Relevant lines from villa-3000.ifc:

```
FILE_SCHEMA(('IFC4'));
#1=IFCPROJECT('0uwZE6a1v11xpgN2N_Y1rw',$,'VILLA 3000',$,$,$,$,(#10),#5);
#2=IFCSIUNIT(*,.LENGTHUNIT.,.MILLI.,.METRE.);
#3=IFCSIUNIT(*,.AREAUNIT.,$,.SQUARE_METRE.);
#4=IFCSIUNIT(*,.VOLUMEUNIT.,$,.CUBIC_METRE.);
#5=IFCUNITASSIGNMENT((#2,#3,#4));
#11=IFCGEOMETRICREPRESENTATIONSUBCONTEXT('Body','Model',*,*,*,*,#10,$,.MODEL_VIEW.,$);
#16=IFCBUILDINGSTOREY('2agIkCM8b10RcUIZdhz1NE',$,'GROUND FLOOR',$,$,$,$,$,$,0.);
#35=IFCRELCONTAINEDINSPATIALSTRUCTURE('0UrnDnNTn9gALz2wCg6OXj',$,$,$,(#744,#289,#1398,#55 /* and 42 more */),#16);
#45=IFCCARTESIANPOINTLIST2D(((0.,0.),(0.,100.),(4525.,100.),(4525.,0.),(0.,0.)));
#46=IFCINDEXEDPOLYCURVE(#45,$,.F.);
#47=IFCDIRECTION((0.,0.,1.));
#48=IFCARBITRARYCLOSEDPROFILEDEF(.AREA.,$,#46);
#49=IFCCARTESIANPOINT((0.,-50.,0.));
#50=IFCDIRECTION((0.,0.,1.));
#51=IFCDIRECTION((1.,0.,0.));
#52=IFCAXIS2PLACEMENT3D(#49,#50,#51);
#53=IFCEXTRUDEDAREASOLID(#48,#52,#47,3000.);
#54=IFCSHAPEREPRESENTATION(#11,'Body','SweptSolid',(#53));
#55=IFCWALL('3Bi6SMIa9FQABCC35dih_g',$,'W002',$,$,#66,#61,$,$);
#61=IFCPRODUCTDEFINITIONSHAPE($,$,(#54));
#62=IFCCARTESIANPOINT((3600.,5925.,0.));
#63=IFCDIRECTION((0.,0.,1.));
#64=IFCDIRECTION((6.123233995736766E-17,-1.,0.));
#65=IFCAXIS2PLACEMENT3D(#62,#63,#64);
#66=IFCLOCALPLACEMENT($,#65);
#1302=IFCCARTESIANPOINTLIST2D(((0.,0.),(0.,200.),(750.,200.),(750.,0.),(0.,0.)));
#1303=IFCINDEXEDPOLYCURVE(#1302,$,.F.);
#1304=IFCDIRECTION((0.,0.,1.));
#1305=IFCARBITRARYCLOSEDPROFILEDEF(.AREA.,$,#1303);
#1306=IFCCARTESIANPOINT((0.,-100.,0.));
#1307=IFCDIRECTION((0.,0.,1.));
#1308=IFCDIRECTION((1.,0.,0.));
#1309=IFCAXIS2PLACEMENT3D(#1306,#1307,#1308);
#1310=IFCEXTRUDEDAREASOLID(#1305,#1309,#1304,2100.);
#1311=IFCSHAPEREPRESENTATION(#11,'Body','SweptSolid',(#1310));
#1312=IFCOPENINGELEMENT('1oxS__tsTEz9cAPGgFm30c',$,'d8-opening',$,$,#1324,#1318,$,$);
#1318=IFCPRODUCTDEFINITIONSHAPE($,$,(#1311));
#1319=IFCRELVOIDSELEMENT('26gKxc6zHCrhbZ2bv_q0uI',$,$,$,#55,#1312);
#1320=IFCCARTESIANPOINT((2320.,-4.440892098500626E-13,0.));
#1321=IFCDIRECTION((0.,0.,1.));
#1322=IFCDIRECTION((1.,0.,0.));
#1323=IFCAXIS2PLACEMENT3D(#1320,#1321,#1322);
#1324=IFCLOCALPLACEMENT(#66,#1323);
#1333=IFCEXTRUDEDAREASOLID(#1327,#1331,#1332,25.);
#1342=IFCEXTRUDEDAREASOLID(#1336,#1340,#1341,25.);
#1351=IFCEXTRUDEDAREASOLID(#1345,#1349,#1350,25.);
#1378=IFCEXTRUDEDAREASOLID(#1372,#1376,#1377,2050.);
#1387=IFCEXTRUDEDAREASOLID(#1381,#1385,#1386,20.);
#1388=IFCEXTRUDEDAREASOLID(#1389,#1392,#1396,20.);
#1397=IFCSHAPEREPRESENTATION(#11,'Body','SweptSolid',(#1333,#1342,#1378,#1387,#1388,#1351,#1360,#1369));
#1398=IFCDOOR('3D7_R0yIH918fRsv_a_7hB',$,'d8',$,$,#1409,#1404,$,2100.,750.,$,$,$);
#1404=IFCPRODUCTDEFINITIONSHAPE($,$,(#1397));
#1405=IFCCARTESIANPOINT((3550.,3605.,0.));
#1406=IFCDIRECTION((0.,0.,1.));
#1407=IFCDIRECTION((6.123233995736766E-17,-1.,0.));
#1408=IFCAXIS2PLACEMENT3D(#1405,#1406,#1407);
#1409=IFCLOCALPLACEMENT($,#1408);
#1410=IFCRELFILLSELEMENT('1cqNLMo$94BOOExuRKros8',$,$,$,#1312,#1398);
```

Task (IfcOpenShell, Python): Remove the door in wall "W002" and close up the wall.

```python
import ifcopenshell
import ifcopenshell.api.feature
import ifcopenshell.api.root
import ifcopenshell.geom
import ifcopenshell.util.shape

model = ifcopenshell.open("villa-3000.ifc")
settings = ifcopenshell.geom.settings()


def volume(element):
    """Net volume in cubic metres, openings subtracted."""
    shape = ifcopenshell.geom.create_shape(settings, element)
    return ifcopenshell.util.shape.get_volume(shape.geometry)


door = model.by_guid("3D7_R0yIH918fRsv_a_7hB")
opening = door.FillsVoids[0].RelatingOpeningElement
wall = opening.VoidsElements[0].RelatingBuildingElement
before = volume(wall)

ifcopenshell.api.root.remove_product(model, product=door)
ifcopenshell.api.feature.remove_feature(model, feature=opening)

after = volume(wall)

print(f"wall volume {before:.3f} -> {after:.3f} m3")

model.write("villa-3000_edited.ifc")
```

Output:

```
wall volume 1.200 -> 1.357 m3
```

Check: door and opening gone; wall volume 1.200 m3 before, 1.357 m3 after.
